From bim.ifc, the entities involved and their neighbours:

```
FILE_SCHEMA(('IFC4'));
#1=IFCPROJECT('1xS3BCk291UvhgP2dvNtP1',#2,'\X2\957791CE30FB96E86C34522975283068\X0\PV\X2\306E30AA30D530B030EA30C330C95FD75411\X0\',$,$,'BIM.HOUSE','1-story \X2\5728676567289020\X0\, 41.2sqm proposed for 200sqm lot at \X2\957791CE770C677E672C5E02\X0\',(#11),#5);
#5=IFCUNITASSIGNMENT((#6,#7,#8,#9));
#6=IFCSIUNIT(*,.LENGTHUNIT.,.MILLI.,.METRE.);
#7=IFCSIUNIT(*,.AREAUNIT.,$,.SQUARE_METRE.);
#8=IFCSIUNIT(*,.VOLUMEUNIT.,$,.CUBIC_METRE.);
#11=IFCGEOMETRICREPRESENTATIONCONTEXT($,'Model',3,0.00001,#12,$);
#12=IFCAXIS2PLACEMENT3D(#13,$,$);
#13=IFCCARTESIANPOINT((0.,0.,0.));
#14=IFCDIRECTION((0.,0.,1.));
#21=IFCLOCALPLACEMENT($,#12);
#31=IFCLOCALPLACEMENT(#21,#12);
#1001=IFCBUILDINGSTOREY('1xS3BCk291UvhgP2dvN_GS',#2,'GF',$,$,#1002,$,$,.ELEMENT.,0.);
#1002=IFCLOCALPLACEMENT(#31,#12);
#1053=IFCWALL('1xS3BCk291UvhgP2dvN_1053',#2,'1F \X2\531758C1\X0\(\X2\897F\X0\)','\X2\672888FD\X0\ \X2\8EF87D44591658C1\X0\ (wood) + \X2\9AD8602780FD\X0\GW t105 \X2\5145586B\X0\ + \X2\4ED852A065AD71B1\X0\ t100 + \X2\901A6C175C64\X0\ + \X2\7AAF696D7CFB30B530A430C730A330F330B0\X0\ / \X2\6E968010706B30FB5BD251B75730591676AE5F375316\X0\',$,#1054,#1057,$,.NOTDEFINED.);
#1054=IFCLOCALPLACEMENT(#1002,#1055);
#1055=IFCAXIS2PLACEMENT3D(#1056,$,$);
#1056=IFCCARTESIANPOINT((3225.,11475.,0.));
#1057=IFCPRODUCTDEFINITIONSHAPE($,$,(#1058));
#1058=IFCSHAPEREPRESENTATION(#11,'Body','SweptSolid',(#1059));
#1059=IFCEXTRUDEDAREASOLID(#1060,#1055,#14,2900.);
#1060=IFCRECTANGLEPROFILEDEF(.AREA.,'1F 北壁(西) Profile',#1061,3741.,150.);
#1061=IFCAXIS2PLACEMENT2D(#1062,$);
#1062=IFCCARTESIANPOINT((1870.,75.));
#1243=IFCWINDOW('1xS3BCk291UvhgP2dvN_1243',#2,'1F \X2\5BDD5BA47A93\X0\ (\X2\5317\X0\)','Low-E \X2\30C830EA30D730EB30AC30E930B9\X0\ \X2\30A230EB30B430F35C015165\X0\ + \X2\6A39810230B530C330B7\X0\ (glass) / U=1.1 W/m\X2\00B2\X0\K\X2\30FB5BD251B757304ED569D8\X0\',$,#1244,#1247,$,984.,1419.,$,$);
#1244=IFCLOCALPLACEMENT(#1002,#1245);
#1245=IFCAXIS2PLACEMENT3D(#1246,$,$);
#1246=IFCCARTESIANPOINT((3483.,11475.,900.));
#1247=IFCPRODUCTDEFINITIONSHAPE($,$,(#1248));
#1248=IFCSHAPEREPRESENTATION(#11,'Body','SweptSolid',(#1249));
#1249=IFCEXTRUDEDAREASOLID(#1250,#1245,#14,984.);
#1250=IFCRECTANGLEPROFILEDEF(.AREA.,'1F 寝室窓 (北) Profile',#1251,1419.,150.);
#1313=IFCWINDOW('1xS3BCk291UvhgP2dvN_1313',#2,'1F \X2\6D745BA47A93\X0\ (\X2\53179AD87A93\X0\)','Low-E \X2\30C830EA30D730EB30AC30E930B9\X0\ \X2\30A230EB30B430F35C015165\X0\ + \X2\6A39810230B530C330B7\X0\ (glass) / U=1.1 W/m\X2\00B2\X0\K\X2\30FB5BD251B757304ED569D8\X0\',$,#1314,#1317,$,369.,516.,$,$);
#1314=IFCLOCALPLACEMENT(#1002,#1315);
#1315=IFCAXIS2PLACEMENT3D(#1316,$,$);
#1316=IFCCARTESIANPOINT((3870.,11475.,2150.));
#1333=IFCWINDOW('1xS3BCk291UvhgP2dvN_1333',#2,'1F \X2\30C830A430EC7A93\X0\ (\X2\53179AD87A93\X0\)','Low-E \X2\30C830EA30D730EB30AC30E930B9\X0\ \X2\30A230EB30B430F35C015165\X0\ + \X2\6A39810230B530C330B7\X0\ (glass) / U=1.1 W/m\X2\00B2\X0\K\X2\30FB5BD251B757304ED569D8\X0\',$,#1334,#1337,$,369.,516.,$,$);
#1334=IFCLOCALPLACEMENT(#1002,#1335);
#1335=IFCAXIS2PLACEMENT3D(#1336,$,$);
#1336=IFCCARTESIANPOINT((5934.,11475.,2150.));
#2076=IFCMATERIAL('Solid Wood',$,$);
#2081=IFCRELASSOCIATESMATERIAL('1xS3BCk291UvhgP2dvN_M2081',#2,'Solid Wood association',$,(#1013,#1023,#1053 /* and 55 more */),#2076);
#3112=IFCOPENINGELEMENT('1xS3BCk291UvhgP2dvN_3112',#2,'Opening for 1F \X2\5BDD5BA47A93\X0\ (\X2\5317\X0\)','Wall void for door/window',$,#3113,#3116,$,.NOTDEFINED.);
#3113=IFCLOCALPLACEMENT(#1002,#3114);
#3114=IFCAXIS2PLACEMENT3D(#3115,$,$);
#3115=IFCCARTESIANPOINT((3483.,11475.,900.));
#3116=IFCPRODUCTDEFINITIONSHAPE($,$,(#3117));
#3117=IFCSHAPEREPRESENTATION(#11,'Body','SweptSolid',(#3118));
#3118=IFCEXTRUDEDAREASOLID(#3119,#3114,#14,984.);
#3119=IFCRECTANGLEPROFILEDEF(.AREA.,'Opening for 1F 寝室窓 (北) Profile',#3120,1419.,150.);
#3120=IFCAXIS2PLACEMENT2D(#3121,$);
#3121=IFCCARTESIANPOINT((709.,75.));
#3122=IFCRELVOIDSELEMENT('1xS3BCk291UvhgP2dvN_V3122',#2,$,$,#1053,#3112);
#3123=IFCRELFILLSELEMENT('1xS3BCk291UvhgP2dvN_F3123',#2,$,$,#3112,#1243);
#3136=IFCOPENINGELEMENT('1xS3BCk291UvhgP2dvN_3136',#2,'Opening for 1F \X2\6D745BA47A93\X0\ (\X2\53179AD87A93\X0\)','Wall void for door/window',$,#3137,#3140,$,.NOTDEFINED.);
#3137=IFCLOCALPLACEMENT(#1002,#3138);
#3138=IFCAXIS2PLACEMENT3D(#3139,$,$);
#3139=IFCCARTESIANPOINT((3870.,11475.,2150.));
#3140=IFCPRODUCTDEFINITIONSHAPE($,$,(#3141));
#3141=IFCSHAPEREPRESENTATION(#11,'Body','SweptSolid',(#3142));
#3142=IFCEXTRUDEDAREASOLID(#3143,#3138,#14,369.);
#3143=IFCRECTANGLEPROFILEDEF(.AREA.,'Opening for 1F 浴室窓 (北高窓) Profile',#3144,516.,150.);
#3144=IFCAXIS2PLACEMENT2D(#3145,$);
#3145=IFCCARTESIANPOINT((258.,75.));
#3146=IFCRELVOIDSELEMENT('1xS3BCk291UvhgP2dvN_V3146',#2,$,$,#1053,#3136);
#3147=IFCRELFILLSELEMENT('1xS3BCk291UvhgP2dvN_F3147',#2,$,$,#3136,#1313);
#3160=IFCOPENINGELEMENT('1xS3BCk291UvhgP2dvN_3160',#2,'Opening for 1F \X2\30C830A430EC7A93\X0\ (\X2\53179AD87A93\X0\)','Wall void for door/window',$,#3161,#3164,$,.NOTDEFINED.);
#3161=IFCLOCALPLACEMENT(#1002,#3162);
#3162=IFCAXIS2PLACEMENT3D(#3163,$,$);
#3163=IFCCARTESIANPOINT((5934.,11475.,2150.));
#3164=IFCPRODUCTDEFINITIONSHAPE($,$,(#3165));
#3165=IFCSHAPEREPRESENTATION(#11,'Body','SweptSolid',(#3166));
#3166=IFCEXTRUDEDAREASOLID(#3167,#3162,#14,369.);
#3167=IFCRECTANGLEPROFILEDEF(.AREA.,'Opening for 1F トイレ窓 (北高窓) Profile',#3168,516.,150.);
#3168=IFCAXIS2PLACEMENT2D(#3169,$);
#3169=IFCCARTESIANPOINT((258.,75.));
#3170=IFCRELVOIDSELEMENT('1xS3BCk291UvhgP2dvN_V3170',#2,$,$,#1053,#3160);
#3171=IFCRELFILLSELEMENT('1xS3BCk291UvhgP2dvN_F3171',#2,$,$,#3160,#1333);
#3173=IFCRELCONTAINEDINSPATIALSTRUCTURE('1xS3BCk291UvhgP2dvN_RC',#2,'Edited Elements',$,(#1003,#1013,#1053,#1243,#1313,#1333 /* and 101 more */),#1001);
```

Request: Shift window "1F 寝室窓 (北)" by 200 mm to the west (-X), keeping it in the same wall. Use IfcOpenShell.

```python
import ifcopenshell
import ifcopenshell.api.geometry
import ifcopenshell.util.placement

model = ifcopenshell.open("bim.ifc")

window = model.by_guid("1xS3BCk291UvhgP2dvN_1243")
opening = window.FillsVoids[0].RelatingOpeningElement
wall = opening.VoidsElements[0].RelatingBuildingElement

wall_matrix = ifcopenshell.util.placement.get_local_placement(wall.ObjectPlacement)
shift = wall_matrix[:3, 0] * -200.0
before = ifcopenshell.util.placement.get_local_placement(window.ObjectPlacement)[:3, 3].copy()

# The window is not placed relative to its opening, so move both.
for product in (opening, window):
    matrix = ifcopenshell.util.placement.get_local_placement(product.ObjectPlacement)
    matrix[:3, 3] += shift
    ifcopenshell.api.geometry.edit_object_placement(model, product=product, matrix=matrix, is_si=False)

after = ifcopenshell.util.placement.get_local_placement(window.ObjectPlacement)[:3, 3]
print("window moved by", (after - before).round(3) + 0.0)

model.write("bim_edited.ifc")
```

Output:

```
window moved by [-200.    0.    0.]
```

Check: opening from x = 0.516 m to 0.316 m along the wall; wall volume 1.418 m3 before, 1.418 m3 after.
